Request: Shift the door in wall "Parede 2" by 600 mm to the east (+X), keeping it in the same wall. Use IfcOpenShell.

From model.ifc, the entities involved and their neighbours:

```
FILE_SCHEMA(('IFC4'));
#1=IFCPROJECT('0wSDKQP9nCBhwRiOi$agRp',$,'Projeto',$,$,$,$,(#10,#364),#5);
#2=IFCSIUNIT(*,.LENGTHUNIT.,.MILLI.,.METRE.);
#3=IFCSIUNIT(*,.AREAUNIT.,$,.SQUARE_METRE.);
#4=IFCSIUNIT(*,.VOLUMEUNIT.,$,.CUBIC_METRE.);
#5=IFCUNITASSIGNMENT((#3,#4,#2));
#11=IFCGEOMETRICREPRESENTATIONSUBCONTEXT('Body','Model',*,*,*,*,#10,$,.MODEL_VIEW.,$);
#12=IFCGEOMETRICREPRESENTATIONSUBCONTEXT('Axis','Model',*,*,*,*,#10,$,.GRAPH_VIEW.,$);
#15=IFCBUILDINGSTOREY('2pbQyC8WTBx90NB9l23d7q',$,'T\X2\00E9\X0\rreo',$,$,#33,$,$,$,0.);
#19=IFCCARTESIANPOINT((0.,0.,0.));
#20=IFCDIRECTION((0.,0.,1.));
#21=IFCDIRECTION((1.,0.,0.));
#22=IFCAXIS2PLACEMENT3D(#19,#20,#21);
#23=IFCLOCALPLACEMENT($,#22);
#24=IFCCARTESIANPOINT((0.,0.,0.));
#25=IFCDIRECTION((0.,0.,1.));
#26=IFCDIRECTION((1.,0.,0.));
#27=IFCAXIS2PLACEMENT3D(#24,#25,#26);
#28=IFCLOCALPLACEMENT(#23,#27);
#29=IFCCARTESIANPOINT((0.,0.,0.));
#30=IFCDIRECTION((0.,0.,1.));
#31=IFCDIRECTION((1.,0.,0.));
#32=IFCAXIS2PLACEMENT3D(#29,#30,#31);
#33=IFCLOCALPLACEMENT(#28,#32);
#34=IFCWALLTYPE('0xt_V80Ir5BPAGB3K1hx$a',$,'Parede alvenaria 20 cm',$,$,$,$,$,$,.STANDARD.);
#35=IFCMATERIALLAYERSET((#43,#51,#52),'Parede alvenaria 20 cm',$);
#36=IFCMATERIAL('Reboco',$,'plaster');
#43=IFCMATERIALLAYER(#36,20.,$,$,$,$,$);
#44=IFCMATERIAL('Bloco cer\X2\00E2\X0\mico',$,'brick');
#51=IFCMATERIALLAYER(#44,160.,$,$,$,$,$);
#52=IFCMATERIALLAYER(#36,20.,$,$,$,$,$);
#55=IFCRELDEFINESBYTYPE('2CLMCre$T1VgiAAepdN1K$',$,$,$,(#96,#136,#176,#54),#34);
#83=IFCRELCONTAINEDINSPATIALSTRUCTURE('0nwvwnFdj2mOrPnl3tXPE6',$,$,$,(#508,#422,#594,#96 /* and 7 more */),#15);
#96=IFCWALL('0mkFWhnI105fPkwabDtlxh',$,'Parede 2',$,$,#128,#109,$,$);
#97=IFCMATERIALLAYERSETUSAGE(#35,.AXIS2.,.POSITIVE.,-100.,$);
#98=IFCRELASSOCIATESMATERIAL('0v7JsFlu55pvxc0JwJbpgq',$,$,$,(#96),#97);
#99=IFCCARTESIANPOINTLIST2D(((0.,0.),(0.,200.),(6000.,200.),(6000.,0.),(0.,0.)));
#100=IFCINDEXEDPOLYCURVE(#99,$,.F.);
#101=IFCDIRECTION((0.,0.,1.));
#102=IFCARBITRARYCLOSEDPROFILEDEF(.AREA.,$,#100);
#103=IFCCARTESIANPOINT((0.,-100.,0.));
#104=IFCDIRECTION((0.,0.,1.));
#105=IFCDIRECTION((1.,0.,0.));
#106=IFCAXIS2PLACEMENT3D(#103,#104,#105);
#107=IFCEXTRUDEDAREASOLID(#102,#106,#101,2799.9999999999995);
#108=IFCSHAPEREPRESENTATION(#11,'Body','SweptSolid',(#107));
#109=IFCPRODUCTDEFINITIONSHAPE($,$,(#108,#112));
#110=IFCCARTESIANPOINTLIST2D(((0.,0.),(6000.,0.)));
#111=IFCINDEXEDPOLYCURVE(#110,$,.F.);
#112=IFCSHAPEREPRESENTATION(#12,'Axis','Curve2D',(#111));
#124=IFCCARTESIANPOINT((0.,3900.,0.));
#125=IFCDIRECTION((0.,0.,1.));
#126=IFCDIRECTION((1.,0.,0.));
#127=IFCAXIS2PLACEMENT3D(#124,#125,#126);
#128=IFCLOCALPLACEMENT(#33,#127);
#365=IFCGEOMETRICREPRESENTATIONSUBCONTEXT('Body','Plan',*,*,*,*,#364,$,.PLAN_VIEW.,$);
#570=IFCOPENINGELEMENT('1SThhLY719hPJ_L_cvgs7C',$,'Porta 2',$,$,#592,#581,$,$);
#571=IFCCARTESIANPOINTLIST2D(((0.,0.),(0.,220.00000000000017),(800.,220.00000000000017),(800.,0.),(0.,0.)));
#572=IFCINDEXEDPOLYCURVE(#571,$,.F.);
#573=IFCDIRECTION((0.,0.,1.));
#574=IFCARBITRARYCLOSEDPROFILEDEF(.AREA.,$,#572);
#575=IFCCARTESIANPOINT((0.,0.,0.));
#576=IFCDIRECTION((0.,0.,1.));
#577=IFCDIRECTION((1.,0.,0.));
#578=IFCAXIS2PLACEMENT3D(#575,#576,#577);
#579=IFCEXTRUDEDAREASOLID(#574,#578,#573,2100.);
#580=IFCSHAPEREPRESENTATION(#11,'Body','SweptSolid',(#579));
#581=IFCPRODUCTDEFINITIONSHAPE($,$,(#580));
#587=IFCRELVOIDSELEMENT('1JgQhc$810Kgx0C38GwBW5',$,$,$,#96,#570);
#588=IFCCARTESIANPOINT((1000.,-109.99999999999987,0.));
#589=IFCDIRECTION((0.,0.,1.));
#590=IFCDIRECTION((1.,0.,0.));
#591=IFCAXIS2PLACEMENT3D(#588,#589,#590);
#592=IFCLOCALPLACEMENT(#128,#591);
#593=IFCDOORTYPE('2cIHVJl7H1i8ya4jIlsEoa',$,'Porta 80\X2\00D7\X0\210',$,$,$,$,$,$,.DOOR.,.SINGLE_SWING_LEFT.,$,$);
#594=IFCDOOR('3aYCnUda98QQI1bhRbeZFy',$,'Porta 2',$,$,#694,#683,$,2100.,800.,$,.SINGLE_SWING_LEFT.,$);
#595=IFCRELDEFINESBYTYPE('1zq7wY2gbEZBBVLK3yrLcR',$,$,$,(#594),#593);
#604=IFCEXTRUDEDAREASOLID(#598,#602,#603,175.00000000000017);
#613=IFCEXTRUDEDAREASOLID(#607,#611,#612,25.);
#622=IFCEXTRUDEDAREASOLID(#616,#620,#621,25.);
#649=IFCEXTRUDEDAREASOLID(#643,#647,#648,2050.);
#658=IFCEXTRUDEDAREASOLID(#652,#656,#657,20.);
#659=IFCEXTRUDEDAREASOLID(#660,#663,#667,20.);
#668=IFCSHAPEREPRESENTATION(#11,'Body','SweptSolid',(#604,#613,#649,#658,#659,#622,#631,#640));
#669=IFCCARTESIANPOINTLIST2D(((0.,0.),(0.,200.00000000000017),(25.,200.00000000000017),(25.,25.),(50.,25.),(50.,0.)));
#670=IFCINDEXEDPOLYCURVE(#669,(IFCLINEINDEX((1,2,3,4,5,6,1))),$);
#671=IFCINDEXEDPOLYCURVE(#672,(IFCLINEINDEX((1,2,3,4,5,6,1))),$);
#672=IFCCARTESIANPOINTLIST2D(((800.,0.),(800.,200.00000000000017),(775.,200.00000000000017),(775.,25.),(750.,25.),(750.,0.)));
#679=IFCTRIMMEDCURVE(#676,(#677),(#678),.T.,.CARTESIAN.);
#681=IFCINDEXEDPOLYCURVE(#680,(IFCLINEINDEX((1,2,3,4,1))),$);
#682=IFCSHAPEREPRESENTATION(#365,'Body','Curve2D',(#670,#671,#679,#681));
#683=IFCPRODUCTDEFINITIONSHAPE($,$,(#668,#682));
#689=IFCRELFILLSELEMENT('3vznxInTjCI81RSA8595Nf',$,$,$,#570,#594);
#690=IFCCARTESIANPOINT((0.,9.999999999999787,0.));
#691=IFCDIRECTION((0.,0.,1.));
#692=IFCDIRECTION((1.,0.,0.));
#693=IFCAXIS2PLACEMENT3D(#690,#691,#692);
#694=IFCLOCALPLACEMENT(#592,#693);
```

```python
import ifcopenshell
import ifcopenshell.api.geometry
import ifcopenshell.util.placement
import ifcopenshell.util.unit

model = ifcopenshell.open("model.ifc")
unit_scale = ifcopenshell.util.unit.calculate_unit_scale(model)

door = model.by_guid("3aYCnUda98QQI1bhRbeZFy")
opening = door.FillsVoids[0].RelatingOpeningElement
wall = opening.VoidsElements[0].RelatingBuildingElement

wall_matrix = ifcopenshell.util.placement.get_local_placement(wall.ObjectPlacement)
shift = wall_matrix[:3, 0] * 0.6 / unit_scale
before = ifcopenshell.util.placement.get_local_placement(door.ObjectPlacement)[:3, 3].copy()

# The door is placed relative to its opening, so it follows when the opening moves.
matrix = ifcopenshell.util.placement.get_local_placement(opening.ObjectPlacement)
matrix[:3, 3] += shift
ifcopenshell.api.geometry.edit_object_placement(
    model, product=opening, matrix=matrix, is_si=False, should_transform_children=True
)

after = ifcopenshell.util.placement.get_local_placement(door.ObjectPlacement)[:3, 3]
print("door moved by", (after - before).round(3) + 0.0)

model.write("model_updated.ifc")
```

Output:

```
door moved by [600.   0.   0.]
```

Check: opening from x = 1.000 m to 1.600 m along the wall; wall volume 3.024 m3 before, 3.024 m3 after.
